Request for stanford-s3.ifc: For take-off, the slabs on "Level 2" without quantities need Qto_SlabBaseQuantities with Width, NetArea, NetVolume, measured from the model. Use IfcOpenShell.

First a look at what the model holds.

```python
import ifcopenshell
import ifcopenshell.util.element
import ifcopenshell.util.unit

model = ifcopenshell.open("stanford-s3.ifc")
print(model.schema)
for unit_type in ("LENGTHUNIT", "AREAUNIT", "VOLUMEUNIT"):
    print(unit_type, ifcopenshell.util.unit.calculate_unit_scale(model, unit_type))
storey = next(s for s in model.by_type("IfcBuildingStorey") if s.Name == "Level 2")
slabs = [e for e in ifcopenshell.util.element.get_decomposition(storey) if e.is_a("IfcSlab")]
for e in sorted(slabs, key=lambda e: e.id()):
    print(e.id(), e.is_a(), e.Name, list(ifcopenshell.util.element.get_psets(e, qtos_only=True)), sep=" | ")
```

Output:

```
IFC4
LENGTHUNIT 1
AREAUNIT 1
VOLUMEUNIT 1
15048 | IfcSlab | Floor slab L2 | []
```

```python
import ifcopenshell
import ifcopenshell.api.pset
import ifcopenshell.geom
import ifcopenshell.util.element
import ifcopenshell.util.shape
import ifcopenshell.util.unit

model = ifcopenshell.open("stanford-s3.ifc")
unit_scale = ifcopenshell.util.unit.calculate_unit_scale(model)
area_scale = ifcopenshell.util.unit.calculate_unit_scale(model, "AREAUNIT")
volume_scale = ifcopenshell.util.unit.calculate_unit_scale(model, "VOLUMEUNIT")
settings = ifcopenshell.geom.settings()

storey = next(s for s in model.by_type("IfcBuildingStorey") if s.Name == "Level 2")
slabs = [e for e in ifcopenshell.util.element.get_decomposition(storey) if e.is_a("IfcSlab")]

for e in sorted(slabs, key=lambda e: e.id()):
    if ifcopenshell.util.element.get_psets(e, qtos_only=True, should_inherit=False):
        continue
    # Geometry comes back in metres, in the element's own axes.
    shape = ifcopenshell.geom.create_shape(settings, e)
    values = {
        "Width": ifcopenshell.util.shape.get_z(shape.geometry) / unit_scale,
        "NetArea": ifcopenshell.util.shape.get_footprint_area(shape.geometry) / area_scale,
        "NetVolume": ifcopenshell.util.shape.get_volume(shape.geometry) / volume_scale,
    }
    qto = ifcopenshell.api.pset.add_qto(model, product=e, name="Qto_SlabBaseQuantities")
    ifcopenshell.api.pset.edit_qto(model, qto=qto, properties=values)
    print(e.id(), {k: round(v, 3) for k, v in values.items()})

model.write("stanford-s3-out.ifc")
```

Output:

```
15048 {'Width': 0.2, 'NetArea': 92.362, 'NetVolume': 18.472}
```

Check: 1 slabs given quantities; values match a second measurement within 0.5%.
